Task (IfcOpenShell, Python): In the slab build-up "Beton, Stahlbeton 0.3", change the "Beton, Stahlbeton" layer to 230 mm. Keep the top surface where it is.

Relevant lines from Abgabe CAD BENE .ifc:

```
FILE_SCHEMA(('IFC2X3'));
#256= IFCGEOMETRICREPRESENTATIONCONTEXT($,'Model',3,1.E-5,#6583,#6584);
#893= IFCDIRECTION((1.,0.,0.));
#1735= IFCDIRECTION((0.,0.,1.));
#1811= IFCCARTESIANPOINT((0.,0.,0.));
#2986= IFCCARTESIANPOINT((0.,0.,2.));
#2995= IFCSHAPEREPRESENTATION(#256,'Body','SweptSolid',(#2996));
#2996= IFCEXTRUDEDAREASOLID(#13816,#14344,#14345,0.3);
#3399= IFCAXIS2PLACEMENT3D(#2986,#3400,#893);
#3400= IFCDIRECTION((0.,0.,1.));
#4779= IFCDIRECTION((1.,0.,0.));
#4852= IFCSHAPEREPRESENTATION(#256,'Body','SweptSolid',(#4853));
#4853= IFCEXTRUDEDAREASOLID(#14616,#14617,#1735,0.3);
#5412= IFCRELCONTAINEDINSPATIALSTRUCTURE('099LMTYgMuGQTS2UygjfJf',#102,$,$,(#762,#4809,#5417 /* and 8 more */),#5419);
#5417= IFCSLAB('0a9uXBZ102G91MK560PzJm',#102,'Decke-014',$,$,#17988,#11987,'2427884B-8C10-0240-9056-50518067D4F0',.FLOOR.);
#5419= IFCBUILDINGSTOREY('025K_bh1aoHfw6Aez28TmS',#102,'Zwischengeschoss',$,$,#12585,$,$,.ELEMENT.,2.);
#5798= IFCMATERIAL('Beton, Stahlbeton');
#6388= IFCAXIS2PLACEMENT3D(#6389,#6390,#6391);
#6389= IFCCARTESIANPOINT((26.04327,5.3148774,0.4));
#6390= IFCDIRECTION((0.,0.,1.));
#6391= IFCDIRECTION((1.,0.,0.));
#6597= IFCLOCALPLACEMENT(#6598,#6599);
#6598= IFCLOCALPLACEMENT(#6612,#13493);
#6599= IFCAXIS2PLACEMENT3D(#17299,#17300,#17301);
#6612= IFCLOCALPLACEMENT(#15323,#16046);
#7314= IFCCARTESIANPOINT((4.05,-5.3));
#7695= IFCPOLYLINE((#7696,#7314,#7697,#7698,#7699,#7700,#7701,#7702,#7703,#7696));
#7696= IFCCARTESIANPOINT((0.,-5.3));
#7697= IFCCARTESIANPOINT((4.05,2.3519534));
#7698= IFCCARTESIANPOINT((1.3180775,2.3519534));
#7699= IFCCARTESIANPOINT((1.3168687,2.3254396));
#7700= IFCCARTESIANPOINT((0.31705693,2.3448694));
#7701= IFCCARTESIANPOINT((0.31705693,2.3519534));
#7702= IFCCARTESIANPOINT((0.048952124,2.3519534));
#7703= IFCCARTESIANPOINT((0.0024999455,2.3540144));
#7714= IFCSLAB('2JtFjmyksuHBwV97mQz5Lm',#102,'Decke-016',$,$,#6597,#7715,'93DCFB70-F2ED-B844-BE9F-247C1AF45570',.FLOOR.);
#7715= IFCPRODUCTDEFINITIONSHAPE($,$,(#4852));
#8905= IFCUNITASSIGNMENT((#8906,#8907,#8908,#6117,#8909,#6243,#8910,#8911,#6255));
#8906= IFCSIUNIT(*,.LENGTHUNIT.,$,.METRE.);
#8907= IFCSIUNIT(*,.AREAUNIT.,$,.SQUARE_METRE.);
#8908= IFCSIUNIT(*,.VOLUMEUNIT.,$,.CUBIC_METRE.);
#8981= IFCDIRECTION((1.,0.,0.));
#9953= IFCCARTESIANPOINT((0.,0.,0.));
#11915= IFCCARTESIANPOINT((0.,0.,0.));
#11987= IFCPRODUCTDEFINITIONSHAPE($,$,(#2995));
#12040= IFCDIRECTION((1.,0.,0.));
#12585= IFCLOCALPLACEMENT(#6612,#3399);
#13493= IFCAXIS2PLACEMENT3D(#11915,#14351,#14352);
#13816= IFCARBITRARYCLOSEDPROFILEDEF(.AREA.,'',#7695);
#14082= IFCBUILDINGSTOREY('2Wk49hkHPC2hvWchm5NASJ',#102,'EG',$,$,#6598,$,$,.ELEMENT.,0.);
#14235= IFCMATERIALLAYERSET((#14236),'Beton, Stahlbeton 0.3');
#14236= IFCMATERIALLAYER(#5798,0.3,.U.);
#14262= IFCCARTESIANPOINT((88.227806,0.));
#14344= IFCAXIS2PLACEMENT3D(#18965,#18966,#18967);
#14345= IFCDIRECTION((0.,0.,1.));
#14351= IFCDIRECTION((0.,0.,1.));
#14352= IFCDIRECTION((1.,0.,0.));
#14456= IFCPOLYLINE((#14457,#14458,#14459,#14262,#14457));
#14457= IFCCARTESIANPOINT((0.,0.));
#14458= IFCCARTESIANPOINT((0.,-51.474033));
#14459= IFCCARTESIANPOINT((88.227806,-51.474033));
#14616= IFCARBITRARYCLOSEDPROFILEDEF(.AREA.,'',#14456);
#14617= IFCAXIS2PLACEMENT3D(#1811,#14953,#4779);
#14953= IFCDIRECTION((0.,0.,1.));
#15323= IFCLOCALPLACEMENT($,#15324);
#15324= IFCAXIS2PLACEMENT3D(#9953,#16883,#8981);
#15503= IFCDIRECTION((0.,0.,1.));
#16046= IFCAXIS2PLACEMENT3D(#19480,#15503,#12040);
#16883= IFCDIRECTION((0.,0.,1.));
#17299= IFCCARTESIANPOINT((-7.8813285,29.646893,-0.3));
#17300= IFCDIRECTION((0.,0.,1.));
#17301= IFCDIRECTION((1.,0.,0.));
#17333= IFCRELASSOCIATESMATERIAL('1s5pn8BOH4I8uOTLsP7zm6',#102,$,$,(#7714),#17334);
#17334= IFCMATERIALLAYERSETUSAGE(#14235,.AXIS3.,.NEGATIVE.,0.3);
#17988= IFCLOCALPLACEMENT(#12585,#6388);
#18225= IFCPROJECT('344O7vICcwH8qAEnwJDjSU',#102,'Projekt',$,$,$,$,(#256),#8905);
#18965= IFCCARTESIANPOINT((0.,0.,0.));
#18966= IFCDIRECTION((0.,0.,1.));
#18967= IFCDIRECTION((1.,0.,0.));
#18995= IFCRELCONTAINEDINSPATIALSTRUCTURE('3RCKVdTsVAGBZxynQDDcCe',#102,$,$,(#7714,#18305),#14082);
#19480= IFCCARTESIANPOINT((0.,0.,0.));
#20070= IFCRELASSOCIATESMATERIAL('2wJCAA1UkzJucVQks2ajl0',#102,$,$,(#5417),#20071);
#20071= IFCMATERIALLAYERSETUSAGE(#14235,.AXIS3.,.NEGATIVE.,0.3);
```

```python
import ifcopenshell
import ifcopenshell.util.element
import ifcopenshell.util.unit

model = ifcopenshell.open("Abgabe CAD BENE .ifc")
unit_scale = ifcopenshell.util.unit.calculate_unit_scale(model)

layer_set = model.by_id(14235)
layer = next(l for l in layer_set.MaterialLayers if l.Material and l.Material.Name == "Beton, Stahlbeton")
change = 0.23 / unit_scale - layer.LayerThickness
layer.LayerThickness += change

# The layer set is shared, so every slab that uses it gets the new thickness.
slabs = [e for e in ifcopenshell.util.element.get_elements_by_material(model, layer_set) if e.is_a("IfcSlab")]
for slab in sorted(slabs, key=lambda e: e.id()):
    body = next(r for r in slab.Representation.Representations if r.RepresentationIdentifier == "Body")
    solid = body.Items[0]
    old_depth = solid.Depth
    solid.Depth += change
    # Extruded upwards: lower the start of the extrusion so the top stays.
    x, y, z = solid.Position.Location.Coordinates
    solid.Position.Location = model.createIfcCartesianPoint((x, y, z - change))
    print(slab.id(), f"{old_depth:g} -> {solid.Depth:g}")

model.write("Abgabe CAD BENE _rev.ifc")
```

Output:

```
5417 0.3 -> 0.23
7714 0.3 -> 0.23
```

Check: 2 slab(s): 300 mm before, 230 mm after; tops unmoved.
